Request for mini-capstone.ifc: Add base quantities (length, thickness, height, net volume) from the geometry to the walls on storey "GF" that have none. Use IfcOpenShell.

First a look at what the model holds.

```python
import ifcopenshell
import ifcopenshell.util.element
import ifcopenshell.util.unit

model = ifcopenshell.open("mini-capstone.ifc")
print(model.schema)
for unit_type in ("LENGTHUNIT", "AREAUNIT", "VOLUMEUNIT"):
    print(unit_type, ifcopenshell.util.unit.calculate_unit_scale(model, unit_type))
storey = next(s for s in model.by_type("IfcBuildingStorey") if s.Name == "GF")
walls = [e for e in ifcopenshell.util.element.get_decomposition(storey) if e.is_a("IfcWall")]
for e in sorted(walls, key=lambda e: e.id()):
    print(e.id(), e.is_a(), e.Name, list(ifcopenshell.util.element.get_psets(e, qtos_only=True)), sep=" | ")
```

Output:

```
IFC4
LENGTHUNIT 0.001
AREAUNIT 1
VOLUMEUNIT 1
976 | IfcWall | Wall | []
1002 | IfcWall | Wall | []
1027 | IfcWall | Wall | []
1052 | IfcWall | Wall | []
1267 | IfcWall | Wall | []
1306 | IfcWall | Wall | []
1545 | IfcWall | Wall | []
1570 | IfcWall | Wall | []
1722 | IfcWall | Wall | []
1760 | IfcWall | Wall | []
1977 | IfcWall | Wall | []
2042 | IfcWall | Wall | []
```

```python
import ifcopenshell
import ifcopenshell.api.pset
import ifcopenshell.geom
import ifcopenshell.util.element
import ifcopenshell.util.shape
import ifcopenshell.util.unit

model = ifcopenshell.open("mini-capstone.ifc")
unit_scale = ifcopenshell.util.unit.calculate_unit_scale(model)
volume_scale = ifcopenshell.util.unit.calculate_unit_scale(model, "VOLUMEUNIT")
settings = ifcopenshell.geom.settings()

storey = next(s for s in model.by_type("IfcBuildingStorey") if s.Name == "GF")
walls = [e for e in ifcopenshell.util.element.get_decomposition(storey) if e.is_a("IfcWall")]

for e in sorted(walls, key=lambda e: e.id()):
    if ifcopenshell.util.element.get_psets(e, qtos_only=True, should_inherit=False):
        continue
    # Geometry comes back in metres, in the element's own axes.
    shape = ifcopenshell.geom.create_shape(settings, e)
    values = {
        "Length": ifcopenshell.util.shape.get_x(shape.geometry) / unit_scale,
        "Width": ifcopenshell.util.shape.get_y(shape.geometry) / unit_scale,
        "Height": ifcopenshell.util.shape.get_z(shape.geometry) / unit_scale,
        "NetVolume": ifcopenshell.util.shape.get_volume(shape.geometry) / volume_scale,
    }
    qto = ifcopenshell.api.pset.add_qto(model, product=e, name="Qto_WallBaseQuantities")
    ifcopenshell.api.pset.edit_qto(model, qto=qto, properties=values)
    print(e.id(), {k: round(v, 3) for k, v in values.items()})

model.write("mini-capstone_rev.ifc")
```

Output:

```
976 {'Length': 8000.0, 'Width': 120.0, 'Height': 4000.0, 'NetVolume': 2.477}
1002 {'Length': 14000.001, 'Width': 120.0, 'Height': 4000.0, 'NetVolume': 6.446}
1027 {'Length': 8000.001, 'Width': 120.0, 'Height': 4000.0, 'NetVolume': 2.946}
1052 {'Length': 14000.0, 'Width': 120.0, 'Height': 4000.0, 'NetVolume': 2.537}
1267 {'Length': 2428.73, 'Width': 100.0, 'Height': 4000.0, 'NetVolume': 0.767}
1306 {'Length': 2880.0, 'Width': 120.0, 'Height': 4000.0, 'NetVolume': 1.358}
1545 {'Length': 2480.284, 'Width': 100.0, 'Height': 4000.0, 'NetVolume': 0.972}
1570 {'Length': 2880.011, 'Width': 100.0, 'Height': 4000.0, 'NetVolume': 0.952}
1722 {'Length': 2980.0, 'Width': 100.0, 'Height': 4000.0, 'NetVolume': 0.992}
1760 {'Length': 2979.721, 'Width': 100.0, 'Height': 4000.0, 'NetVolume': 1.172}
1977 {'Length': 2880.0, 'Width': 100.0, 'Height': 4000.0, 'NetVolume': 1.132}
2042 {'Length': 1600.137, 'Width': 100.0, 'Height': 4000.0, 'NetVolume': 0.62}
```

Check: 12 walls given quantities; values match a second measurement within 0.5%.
